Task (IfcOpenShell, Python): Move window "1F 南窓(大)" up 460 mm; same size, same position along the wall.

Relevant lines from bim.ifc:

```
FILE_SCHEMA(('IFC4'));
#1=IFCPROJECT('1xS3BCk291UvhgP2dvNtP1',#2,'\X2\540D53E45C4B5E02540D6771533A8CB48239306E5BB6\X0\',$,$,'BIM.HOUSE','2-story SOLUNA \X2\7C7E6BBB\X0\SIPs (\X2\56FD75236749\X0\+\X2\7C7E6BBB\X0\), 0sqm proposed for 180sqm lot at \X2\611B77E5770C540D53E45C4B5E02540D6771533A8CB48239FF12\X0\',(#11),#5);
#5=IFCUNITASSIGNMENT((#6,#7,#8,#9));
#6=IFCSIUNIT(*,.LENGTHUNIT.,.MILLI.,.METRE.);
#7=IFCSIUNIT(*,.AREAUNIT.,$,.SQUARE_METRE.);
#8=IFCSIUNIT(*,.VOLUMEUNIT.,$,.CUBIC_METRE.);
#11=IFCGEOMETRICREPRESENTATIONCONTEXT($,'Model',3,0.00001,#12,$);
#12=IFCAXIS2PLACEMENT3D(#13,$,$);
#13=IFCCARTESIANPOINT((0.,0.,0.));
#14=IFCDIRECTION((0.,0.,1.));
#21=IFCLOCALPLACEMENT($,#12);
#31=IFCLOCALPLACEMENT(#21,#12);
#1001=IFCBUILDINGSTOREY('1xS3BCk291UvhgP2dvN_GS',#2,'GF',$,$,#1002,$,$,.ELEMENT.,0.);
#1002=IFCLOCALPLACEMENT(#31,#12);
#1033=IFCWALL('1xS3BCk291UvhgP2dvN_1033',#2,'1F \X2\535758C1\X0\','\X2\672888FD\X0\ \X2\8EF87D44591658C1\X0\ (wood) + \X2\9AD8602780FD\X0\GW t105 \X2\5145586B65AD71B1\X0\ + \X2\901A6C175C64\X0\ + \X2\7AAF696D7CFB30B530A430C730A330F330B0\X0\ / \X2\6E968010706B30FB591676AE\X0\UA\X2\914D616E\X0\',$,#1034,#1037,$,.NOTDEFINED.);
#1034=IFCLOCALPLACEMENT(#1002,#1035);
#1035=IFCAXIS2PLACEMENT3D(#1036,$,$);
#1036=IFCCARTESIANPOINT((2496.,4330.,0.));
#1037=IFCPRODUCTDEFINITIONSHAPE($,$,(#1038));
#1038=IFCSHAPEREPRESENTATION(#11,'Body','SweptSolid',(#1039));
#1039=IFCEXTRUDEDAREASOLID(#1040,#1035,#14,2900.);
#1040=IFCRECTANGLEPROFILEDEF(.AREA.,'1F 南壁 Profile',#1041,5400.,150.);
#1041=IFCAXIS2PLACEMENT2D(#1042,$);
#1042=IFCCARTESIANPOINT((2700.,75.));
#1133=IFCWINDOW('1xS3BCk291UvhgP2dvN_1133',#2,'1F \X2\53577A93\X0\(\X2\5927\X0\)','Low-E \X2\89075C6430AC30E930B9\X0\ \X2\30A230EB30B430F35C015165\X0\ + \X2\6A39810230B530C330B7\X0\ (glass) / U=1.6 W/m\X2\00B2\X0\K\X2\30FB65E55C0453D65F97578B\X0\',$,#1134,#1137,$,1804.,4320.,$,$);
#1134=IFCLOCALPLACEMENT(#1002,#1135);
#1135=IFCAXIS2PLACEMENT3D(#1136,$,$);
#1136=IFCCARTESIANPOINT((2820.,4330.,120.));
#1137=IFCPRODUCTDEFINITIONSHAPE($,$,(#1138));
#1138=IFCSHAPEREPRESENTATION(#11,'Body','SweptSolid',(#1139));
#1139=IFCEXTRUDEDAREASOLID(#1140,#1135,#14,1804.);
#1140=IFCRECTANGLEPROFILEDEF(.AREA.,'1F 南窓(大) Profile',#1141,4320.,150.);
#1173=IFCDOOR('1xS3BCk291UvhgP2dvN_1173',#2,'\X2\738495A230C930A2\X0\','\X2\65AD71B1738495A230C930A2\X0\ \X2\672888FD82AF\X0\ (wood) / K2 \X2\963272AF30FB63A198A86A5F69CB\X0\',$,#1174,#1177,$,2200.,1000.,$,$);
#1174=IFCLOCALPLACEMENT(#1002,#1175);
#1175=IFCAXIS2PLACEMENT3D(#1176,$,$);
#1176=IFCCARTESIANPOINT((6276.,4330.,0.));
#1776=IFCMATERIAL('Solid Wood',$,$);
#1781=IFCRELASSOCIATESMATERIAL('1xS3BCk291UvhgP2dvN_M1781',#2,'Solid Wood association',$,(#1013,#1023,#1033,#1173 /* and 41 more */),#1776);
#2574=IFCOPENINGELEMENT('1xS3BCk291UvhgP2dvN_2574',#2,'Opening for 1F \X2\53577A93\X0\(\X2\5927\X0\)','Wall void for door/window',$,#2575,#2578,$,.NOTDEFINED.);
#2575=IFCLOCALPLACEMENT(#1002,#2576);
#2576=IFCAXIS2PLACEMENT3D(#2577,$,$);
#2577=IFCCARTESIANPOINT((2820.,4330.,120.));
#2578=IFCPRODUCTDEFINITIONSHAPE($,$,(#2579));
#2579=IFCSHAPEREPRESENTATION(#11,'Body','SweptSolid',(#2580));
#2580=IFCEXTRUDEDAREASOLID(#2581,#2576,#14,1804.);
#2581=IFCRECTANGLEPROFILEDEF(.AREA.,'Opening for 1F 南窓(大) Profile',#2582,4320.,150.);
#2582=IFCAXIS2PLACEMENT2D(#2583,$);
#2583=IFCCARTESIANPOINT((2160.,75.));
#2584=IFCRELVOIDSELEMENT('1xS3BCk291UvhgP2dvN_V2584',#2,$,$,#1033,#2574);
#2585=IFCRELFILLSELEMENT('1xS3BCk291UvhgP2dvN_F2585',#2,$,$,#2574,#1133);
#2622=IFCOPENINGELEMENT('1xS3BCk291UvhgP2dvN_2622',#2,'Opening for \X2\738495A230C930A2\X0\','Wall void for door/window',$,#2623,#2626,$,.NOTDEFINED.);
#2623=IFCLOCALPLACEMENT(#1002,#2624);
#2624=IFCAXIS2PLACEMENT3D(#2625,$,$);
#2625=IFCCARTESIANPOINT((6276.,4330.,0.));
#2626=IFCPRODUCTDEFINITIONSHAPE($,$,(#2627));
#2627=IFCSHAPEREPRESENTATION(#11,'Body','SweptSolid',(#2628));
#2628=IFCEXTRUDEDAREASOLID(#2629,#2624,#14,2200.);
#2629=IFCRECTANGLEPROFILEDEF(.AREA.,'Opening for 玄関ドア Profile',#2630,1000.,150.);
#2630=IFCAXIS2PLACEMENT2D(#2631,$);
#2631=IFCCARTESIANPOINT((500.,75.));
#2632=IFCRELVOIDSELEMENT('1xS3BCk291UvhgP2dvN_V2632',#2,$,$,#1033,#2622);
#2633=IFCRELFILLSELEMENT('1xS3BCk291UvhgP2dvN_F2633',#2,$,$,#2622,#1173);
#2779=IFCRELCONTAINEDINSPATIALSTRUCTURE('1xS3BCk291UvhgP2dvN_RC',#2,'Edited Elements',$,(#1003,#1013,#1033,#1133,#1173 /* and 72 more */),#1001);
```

```python
import numpy as np
import ifcopenshell
import ifcopenshell.api.geometry
import ifcopenshell.util.placement
import ifcopenshell.util.unit

model = ifcopenshell.open("bim.ifc")
unit_scale = ifcopenshell.util.unit.calculate_unit_scale(model)

window = model.by_guid("1xS3BCk291UvhgP2dvN_1133")
opening = window.FillsVoids[0].RelatingOpeningElement
dz = 0.46 / unit_scale

shift = np.array([0.0, 0.0, dz])
# The window is not placed relative to its opening, so move both.
for product in (opening, window):
    matrix = ifcopenshell.util.placement.get_local_placement(product.ObjectPlacement)
    matrix[:3, 3] += shift
    ifcopenshell.api.geometry.edit_object_placement(model, product=product, matrix=matrix, is_si=False)

print(f"moved by {dz * unit_scale:+.3f} m")

model.write("bim_edited.ifc")
```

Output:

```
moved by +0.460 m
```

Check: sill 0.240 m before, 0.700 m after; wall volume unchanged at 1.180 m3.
